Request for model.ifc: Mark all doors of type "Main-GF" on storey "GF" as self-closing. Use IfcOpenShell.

First a look at what the model holds.

```python
import ifcopenshell
import ifcopenshell.util.element

model = ifcopenshell.open("model.ifc")
print(model.schema)
storey = next(s for s in model.by_type("IfcBuildingStorey") if s.Name == "GF")
doors = [e for e in ifcopenshell.util.element.get_decomposition(storey) if e.is_a("IfcDoor")]
seen = {}
for e in doors:
    element_type = ifcopenshell.util.element.get_type(e)
    key = (element_type.Name if element_type != e and element_type else None, ifcopenshell.util.element.get_pset(e, "Pset_DoorCommon", "SelfClosing"))
    seen[key] = seen.get(key, 0) + 1
for (name, value), count in sorted(seen.items(), key=str):
    print(count, "x", name, "|", value)
```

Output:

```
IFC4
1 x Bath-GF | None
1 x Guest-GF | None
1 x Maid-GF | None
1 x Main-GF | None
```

```python
import ifcopenshell
import ifcopenshell.api.pset
import ifcopenshell.util.element

model = ifcopenshell.open("model.ifc")

storey = next(s for s in model.by_type("IfcBuildingStorey") if s.Name == "GF")
doors = [e for e in ifcopenshell.util.element.get_decomposition(storey) if e.is_a("IfcDoor")]

count = 0
for e in doors:
    element_type = ifcopenshell.util.element.get_type(e)
    if element_type in (None, e) or element_type.Name != "Main-GF":
        continue
    # add_pset returns the element's existing set when there is one.
    pset = ifcopenshell.api.pset.add_pset(model, product=e, name="Pset_DoorCommon")
    ifcopenshell.api.pset.edit_pset(model, pset=pset, properties={"SelfClosing": True})
    count += 1

print(count, "doors updated")

model.write("model_rev.ifc")
```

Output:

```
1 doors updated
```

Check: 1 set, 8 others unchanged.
